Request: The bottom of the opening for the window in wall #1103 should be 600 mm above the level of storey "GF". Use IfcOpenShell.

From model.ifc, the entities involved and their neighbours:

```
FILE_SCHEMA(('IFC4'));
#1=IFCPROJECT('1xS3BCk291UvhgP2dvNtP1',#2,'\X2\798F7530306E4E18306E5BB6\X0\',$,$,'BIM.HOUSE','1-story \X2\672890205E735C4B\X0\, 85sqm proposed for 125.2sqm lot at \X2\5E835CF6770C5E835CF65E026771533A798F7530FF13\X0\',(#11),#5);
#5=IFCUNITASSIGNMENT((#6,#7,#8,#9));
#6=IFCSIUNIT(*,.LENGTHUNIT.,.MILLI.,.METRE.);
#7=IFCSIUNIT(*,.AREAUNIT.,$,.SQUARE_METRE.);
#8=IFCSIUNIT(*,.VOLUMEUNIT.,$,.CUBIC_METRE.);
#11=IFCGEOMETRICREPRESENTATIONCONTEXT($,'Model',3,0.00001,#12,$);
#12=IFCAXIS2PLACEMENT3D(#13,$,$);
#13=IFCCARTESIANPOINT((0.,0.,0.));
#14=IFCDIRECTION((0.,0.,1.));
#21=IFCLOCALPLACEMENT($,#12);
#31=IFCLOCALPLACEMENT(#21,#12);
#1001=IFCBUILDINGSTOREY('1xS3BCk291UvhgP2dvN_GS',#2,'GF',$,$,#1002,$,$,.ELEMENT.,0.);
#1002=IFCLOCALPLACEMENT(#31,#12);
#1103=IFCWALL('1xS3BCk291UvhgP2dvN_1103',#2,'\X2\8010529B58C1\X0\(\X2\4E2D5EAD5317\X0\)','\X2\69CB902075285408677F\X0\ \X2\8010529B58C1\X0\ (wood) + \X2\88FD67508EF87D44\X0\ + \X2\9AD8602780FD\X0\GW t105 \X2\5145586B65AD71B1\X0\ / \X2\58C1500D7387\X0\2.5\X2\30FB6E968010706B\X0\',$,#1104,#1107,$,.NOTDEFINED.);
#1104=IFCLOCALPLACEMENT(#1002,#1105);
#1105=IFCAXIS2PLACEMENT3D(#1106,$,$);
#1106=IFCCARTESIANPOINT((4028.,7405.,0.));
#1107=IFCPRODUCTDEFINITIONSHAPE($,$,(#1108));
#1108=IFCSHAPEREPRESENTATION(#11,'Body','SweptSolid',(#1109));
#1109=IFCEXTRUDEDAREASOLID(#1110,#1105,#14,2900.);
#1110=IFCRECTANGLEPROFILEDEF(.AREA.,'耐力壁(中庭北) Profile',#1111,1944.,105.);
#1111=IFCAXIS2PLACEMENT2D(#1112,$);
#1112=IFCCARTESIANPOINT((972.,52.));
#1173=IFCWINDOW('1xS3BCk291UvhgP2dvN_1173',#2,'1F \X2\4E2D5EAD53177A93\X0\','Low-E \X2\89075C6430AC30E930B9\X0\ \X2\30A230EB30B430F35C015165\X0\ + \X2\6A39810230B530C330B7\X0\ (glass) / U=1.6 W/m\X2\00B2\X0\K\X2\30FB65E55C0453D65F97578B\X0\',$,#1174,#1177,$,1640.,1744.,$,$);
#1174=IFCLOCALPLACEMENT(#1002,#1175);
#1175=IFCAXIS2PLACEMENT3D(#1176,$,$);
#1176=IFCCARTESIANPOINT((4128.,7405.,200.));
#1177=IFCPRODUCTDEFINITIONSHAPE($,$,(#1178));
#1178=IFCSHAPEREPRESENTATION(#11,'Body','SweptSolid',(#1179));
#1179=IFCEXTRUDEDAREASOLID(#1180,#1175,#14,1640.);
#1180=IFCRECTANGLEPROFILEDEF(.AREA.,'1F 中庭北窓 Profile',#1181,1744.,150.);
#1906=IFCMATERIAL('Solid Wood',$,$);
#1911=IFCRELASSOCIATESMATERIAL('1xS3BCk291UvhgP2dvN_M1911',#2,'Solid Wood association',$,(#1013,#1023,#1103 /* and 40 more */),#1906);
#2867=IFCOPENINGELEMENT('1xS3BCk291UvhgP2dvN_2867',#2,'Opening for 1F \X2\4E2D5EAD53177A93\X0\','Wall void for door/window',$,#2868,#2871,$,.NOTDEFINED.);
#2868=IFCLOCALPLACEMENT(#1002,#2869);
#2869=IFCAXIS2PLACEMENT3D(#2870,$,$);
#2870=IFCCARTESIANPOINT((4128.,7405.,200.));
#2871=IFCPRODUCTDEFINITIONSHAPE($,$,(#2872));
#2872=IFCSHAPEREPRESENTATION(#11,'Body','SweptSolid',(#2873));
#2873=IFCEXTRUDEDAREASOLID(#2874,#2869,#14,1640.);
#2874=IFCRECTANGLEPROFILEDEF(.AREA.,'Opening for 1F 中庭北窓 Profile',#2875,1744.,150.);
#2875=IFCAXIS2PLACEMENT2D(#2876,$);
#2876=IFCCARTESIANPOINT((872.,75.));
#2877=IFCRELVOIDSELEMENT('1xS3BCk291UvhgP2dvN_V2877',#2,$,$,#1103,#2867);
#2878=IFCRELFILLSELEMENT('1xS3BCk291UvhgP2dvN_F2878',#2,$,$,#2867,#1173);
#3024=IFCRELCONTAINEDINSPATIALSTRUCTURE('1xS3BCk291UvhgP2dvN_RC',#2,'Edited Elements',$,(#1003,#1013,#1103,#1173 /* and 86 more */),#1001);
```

```python
import numpy as np
import ifcopenshell
import ifcopenshell.api.geometry
import ifcopenshell.geom
import ifcopenshell.util.element
import ifcopenshell.util.placement
import ifcopenshell.util.shape
import ifcopenshell.util.unit

model = ifcopenshell.open("model.ifc")
unit_scale = ifcopenshell.util.unit.calculate_unit_scale(model)

window = model.by_guid("1xS3BCk291UvhgP2dvN_1173")
opening = window.FillsVoids[0].RelatingOpeningElement
storey = ifcopenshell.util.element.get_container(window, ifc_class="IfcBuildingStorey")
level = ifcopenshell.util.placement.get_local_placement(storey.ObjectPlacement)[2, 3]

# The opening's origin need not be at the sill, so measure its lowest point.
shape = ifcopenshell.geom.create_shape(ifcopenshell.geom.settings(), opening)
bottom = ifcopenshell.util.shape.get_shape_bottom_elevation(shape, shape.geometry) / unit_scale
dz = level + 600.0 - bottom

shift = np.array([0.0, 0.0, dz])
# The window is not placed relative to its opening, so move both.
for product in (opening, window):
    matrix = ifcopenshell.util.placement.get_local_placement(product.ObjectPlacement)
    matrix[:3, 3] += shift
    ifcopenshell.api.geometry.edit_object_placement(model, product=product, matrix=matrix, is_si=False)

print(f"moved by {dz * unit_scale:+.3f} m")

model.write("model_rev.ifc")
```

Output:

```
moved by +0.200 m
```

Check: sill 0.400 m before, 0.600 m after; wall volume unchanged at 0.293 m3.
